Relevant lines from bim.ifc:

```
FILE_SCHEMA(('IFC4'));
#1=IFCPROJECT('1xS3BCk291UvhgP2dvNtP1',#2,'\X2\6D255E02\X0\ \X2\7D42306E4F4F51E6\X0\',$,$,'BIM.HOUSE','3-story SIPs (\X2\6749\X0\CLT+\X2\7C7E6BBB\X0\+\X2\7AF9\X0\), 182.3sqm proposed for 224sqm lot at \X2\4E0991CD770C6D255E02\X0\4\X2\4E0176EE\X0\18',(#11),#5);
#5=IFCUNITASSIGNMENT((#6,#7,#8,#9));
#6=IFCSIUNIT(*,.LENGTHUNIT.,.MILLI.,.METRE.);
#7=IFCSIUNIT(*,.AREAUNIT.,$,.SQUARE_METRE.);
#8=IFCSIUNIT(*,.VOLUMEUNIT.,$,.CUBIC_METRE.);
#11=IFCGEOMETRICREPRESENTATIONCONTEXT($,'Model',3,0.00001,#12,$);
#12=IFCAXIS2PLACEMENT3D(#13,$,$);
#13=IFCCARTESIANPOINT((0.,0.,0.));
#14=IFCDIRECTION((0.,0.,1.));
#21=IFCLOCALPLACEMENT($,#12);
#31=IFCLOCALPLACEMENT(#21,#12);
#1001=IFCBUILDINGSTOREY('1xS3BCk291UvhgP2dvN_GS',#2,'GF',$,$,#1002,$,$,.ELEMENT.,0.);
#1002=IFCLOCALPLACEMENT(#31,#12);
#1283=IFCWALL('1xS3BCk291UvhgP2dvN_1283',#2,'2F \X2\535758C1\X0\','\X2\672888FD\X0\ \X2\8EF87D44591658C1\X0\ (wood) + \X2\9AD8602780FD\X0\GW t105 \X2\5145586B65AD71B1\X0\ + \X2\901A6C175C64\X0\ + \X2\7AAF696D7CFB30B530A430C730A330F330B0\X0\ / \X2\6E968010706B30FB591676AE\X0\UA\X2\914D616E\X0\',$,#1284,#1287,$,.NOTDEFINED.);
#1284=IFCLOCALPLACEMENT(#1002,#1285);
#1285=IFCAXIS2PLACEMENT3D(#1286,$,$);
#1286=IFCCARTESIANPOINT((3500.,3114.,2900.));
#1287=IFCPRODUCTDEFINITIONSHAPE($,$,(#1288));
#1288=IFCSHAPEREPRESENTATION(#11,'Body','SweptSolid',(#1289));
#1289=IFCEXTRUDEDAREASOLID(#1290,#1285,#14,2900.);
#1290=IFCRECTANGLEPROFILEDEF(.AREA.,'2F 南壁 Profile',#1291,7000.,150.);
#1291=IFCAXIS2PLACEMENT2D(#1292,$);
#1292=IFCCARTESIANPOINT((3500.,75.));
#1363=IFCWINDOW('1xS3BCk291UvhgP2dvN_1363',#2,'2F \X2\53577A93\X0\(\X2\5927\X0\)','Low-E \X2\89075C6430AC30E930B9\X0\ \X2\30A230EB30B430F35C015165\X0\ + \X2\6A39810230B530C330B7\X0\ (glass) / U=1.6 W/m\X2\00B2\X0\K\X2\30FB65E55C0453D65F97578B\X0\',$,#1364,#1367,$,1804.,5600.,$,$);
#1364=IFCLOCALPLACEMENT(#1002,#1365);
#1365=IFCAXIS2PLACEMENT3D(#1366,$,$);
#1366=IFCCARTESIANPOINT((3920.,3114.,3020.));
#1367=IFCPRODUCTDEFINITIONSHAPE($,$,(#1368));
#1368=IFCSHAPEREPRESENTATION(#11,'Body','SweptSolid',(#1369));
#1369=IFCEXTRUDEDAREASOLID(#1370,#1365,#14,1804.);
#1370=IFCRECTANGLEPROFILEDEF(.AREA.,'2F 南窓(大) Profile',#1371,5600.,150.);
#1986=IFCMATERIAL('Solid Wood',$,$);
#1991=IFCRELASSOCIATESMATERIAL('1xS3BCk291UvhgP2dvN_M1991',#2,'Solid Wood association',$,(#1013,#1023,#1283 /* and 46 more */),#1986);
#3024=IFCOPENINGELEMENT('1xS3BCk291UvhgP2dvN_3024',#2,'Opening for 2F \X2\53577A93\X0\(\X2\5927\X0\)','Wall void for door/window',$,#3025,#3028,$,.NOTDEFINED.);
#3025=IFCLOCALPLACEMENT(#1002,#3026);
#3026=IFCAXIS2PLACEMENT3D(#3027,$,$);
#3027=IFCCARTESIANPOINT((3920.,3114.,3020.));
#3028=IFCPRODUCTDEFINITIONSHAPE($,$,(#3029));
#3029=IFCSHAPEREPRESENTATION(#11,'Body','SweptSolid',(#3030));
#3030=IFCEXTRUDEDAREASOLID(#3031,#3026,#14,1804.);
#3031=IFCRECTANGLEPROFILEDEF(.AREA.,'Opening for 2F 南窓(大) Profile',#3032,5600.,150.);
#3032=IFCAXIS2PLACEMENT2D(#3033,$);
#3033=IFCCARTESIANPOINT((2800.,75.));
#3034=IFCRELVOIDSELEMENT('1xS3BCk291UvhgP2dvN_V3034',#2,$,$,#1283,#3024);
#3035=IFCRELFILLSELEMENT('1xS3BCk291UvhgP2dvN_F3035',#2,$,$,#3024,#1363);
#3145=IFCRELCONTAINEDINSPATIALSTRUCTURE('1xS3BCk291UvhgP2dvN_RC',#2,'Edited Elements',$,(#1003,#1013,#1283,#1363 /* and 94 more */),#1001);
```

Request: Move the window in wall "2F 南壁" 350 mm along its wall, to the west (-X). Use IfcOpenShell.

```python
import ifcopenshell
import ifcopenshell.api.geometry
import ifcopenshell.util.placement

model = ifcopenshell.open("bim.ifc")

window = model.by_guid("1xS3BCk291UvhgP2dvN_1363")
opening = window.FillsVoids[0].RelatingOpeningElement
wall = opening.VoidsElements[0].RelatingBuildingElement

wall_matrix = ifcopenshell.util.placement.get_local_placement(wall.ObjectPlacement)
shift = wall_matrix[:3, 0] * -350.0
before = ifcopenshell.util.placement.get_local_placement(window.ObjectPlacement)[:3, 3].copy()

# The window is not placed relative to its opening, so move both.
for product in (opening, window):
    matrix = ifcopenshell.util.placement.get_local_placement(product.ObjectPlacement)
    matrix[:3, 3] += shift
    ifcopenshell.api.geometry.edit_object_placement(model, product=product, matrix=matrix, is_si=False)

after = ifcopenshell.util.placement.get_local_placement(window.ObjectPlacement)[:3, 3]
print("window moved by", (after - before).round(3) + 0.0)

model.write("bim_v2.ifc")
```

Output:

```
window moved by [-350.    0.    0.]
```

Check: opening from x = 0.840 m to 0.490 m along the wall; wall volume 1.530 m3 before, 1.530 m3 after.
